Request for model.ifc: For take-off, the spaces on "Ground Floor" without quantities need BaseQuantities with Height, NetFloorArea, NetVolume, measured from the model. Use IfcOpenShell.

First a look at what the model holds.

```python
import ifcopenshell
import ifcopenshell.util.element
import ifcopenshell.util.unit

model = ifcopenshell.open("model.ifc")
print(model.schema)
for unit_type in ("LENGTHUNIT", "AREAUNIT", "VOLUMEUNIT"):
    print(unit_type, ifcopenshell.util.unit.calculate_unit_scale(model, unit_type))
storey = next(s for s in model.by_type("IfcBuildingStorey") if s.Name == "Ground Floor")
spaces = [e for e in ifcopenshell.util.element.get_decomposition(storey) if e.is_a("IfcSpace")]
for e in sorted(spaces, key=lambda e: e.id()):
    print(e.id(), e.is_a(), e.Name, list(ifcopenshell.util.element.get_psets(e, qtos_only=True)), sep=" | ")
```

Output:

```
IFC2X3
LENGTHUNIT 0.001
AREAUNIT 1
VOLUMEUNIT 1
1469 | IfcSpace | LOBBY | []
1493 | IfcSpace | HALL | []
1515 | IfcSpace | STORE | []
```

```python
import ifcopenshell
import ifcopenshell.api.pset
import ifcopenshell.geom
import ifcopenshell.util.element
import ifcopenshell.util.shape
import ifcopenshell.util.unit

model = ifcopenshell.open("model.ifc")
unit_scale = ifcopenshell.util.unit.calculate_unit_scale(model)
area_scale = ifcopenshell.util.unit.calculate_unit_scale(model, "AREAUNIT")
volume_scale = ifcopenshell.util.unit.calculate_unit_scale(model, "VOLUMEUNIT")
settings = ifcopenshell.geom.settings()

storey = next(s for s in model.by_type("IfcBuildingStorey") if s.Name == "Ground Floor")
spaces = [e for e in ifcopenshell.util.element.get_decomposition(storey) if e.is_a("IfcSpace")]

for e in sorted(spaces, key=lambda e: e.id()):
    if ifcopenshell.util.element.get_psets(e, qtos_only=True, should_inherit=False):
        continue
    # Geometry comes back in metres, in the element's own axes.
    shape = ifcopenshell.geom.create_shape(settings, e)
    values = {
        "Height": ifcopenshell.util.shape.get_z(shape.geometry) / unit_scale,
        "NetFloorArea": ifcopenshell.util.shape.get_footprint_area(shape.geometry) / area_scale,
        "NetVolume": ifcopenshell.util.shape.get_volume(shape.geometry) / volume_scale,
    }
    qto = ifcopenshell.api.pset.add_qto(model, product=e, name="BaseQuantities")
    ifcopenshell.api.pset.edit_qto(model, qto=qto, properties=values)
    print(e.id(), {k: round(v, 3) for k, v in values.items()})

model.write("model_v2.ifc")
```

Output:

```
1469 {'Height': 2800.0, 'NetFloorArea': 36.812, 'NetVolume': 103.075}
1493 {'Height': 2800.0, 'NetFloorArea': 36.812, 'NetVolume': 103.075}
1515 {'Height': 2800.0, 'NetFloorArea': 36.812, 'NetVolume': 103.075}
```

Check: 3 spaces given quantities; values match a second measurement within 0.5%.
